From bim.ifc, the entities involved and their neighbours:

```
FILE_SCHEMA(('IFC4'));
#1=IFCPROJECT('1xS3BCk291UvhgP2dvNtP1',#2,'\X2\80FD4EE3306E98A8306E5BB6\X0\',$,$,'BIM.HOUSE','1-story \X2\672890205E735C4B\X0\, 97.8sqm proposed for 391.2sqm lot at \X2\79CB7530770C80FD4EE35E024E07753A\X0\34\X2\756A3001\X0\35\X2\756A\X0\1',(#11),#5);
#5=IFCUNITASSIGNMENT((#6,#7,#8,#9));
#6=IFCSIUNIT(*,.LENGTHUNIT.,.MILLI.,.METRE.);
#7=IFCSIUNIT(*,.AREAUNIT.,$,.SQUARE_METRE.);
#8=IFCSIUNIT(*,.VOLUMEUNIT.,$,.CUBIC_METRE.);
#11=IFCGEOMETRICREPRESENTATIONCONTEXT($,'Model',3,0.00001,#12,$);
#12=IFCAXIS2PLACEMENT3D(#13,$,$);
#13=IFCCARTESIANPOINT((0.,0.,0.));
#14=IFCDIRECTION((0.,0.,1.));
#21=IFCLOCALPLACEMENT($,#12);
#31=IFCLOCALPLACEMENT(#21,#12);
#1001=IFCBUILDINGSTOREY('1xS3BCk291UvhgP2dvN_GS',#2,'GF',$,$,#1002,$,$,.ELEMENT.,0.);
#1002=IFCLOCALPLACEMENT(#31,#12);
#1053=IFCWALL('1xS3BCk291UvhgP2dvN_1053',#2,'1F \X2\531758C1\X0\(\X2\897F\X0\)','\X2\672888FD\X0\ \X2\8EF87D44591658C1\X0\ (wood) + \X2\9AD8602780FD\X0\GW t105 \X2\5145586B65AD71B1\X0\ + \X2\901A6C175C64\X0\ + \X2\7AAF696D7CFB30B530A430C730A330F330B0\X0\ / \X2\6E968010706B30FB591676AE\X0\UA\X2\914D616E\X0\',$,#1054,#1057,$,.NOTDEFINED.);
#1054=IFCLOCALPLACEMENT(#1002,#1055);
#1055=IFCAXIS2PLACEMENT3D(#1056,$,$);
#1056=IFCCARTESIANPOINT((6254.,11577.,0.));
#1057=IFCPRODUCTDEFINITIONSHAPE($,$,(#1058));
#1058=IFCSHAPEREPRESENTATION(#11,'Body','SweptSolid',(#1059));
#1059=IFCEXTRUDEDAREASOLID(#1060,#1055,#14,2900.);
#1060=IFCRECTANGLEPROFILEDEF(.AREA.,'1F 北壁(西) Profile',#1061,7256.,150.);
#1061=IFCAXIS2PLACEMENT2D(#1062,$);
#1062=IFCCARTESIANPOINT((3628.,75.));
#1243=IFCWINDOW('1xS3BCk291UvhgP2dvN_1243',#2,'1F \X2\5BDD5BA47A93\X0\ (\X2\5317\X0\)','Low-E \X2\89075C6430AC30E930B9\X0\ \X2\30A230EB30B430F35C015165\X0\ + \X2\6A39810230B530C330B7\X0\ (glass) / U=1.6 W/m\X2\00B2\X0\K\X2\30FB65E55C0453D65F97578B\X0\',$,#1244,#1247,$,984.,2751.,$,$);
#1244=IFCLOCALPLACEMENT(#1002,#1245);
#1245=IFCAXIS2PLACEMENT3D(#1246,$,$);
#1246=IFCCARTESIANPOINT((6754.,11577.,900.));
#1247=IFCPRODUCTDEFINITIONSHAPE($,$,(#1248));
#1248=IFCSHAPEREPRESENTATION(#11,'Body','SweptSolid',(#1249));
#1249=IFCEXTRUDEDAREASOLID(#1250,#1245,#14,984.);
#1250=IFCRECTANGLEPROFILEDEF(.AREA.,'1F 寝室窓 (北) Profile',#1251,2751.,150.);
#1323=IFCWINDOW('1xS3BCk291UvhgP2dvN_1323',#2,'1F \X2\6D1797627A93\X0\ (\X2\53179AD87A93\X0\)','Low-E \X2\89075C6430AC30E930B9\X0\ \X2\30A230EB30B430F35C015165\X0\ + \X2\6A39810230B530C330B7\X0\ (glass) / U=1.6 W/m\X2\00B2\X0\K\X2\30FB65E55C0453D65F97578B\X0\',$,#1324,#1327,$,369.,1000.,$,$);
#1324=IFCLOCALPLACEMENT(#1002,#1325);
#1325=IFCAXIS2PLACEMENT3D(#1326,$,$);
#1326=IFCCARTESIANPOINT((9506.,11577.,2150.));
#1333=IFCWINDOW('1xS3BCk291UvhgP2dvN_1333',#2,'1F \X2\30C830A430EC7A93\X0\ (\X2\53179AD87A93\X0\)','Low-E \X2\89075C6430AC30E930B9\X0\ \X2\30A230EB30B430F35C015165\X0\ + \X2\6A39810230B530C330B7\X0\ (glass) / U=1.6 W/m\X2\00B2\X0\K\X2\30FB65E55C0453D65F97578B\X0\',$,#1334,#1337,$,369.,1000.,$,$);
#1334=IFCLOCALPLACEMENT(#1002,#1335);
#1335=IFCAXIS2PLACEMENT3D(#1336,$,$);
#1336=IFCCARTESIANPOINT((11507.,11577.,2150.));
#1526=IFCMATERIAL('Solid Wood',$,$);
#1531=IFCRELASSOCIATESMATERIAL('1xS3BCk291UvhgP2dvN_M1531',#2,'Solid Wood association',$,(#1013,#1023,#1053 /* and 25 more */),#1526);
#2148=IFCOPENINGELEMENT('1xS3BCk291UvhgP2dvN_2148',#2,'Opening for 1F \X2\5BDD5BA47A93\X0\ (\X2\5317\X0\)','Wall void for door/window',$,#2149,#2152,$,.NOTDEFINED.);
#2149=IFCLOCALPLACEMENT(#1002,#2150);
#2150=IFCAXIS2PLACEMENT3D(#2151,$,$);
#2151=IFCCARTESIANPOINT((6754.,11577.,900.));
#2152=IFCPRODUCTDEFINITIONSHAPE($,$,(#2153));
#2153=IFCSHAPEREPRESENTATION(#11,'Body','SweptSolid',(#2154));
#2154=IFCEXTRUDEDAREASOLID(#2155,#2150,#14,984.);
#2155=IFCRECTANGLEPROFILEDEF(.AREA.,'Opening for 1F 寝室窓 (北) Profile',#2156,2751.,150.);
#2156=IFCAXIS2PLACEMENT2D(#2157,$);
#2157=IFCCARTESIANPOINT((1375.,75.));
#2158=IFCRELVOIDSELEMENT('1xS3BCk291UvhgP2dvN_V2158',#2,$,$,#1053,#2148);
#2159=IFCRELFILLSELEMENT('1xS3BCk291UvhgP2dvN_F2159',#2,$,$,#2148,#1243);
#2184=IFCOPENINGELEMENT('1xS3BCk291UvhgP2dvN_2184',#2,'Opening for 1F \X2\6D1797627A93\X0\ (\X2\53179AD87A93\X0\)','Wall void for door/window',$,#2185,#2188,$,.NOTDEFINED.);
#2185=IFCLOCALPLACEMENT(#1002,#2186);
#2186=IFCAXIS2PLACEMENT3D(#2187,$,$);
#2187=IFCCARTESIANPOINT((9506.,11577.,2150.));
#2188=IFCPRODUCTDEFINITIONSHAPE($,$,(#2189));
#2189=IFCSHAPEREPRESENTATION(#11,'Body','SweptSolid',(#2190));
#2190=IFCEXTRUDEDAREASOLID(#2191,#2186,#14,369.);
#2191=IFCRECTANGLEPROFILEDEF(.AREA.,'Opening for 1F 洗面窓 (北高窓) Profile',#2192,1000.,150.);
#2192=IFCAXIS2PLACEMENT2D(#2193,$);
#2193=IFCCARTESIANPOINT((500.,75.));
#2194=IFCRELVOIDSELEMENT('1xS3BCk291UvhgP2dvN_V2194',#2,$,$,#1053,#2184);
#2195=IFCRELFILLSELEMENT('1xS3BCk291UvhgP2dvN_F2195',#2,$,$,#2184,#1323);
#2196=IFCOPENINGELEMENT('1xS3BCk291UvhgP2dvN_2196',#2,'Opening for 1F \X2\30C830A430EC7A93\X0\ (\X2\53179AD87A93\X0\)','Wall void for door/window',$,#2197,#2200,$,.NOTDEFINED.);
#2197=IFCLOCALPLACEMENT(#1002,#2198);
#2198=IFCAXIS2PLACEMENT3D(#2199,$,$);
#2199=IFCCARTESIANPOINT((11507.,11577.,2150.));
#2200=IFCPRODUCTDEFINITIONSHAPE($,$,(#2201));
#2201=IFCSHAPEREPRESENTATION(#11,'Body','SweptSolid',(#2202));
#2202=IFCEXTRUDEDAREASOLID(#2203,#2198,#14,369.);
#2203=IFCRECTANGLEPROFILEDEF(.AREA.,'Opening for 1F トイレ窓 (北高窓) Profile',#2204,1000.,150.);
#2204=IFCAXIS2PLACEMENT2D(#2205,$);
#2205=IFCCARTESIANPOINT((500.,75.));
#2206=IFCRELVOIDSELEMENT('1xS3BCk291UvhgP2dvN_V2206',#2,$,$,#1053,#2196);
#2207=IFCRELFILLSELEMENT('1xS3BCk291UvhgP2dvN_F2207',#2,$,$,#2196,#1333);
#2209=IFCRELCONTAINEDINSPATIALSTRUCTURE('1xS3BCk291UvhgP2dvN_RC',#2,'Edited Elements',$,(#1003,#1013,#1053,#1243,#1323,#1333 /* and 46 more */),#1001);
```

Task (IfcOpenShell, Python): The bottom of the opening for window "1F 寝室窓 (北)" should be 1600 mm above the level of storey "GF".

```python
import numpy as np
import ifcopenshell
import ifcopenshell.api.geometry
import ifcopenshell.geom
import ifcopenshell.util.element
import ifcopenshell.util.placement
import ifcopenshell.util.shape
import ifcopenshell.util.unit

model = ifcopenshell.open("bim.ifc")
unit_scale = ifcopenshell.util.unit.calculate_unit_scale(model)

window = model.by_id(1243)
opening = window.FillsVoids[0].RelatingOpeningElement
storey = ifcopenshell.util.element.get_container(window, ifc_class="IfcBuildingStorey")
level = ifcopenshell.util.placement.get_local_placement(storey.ObjectPlacement)[2, 3]

# The opening's origin need not be at the sill, so measure its lowest point.
shape = ifcopenshell.geom.create_shape(ifcopenshell.geom.settings(), opening)
bottom = ifcopenshell.util.shape.get_shape_bottom_elevation(shape, shape.geometry) / unit_scale
dz = level + 1.6 / unit_scale - bottom

shift = np.array([0.0, 0.0, dz])
# The window is not placed relative to its opening, so move both.
for product in (opening, window):
    matrix = ifcopenshell.util.placement.get_local_placement(product.ObjectPlacement)
    matrix[:3, 3] += shift
    ifcopenshell.api.geometry.edit_object_placement(model, product=product, matrix=matrix, is_si=False)

print(f"moved by {dz * unit_scale:+.3f} m")

model.write("bim_v2.ifc")
```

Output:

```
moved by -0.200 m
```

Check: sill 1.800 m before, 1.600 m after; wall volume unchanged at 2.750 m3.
